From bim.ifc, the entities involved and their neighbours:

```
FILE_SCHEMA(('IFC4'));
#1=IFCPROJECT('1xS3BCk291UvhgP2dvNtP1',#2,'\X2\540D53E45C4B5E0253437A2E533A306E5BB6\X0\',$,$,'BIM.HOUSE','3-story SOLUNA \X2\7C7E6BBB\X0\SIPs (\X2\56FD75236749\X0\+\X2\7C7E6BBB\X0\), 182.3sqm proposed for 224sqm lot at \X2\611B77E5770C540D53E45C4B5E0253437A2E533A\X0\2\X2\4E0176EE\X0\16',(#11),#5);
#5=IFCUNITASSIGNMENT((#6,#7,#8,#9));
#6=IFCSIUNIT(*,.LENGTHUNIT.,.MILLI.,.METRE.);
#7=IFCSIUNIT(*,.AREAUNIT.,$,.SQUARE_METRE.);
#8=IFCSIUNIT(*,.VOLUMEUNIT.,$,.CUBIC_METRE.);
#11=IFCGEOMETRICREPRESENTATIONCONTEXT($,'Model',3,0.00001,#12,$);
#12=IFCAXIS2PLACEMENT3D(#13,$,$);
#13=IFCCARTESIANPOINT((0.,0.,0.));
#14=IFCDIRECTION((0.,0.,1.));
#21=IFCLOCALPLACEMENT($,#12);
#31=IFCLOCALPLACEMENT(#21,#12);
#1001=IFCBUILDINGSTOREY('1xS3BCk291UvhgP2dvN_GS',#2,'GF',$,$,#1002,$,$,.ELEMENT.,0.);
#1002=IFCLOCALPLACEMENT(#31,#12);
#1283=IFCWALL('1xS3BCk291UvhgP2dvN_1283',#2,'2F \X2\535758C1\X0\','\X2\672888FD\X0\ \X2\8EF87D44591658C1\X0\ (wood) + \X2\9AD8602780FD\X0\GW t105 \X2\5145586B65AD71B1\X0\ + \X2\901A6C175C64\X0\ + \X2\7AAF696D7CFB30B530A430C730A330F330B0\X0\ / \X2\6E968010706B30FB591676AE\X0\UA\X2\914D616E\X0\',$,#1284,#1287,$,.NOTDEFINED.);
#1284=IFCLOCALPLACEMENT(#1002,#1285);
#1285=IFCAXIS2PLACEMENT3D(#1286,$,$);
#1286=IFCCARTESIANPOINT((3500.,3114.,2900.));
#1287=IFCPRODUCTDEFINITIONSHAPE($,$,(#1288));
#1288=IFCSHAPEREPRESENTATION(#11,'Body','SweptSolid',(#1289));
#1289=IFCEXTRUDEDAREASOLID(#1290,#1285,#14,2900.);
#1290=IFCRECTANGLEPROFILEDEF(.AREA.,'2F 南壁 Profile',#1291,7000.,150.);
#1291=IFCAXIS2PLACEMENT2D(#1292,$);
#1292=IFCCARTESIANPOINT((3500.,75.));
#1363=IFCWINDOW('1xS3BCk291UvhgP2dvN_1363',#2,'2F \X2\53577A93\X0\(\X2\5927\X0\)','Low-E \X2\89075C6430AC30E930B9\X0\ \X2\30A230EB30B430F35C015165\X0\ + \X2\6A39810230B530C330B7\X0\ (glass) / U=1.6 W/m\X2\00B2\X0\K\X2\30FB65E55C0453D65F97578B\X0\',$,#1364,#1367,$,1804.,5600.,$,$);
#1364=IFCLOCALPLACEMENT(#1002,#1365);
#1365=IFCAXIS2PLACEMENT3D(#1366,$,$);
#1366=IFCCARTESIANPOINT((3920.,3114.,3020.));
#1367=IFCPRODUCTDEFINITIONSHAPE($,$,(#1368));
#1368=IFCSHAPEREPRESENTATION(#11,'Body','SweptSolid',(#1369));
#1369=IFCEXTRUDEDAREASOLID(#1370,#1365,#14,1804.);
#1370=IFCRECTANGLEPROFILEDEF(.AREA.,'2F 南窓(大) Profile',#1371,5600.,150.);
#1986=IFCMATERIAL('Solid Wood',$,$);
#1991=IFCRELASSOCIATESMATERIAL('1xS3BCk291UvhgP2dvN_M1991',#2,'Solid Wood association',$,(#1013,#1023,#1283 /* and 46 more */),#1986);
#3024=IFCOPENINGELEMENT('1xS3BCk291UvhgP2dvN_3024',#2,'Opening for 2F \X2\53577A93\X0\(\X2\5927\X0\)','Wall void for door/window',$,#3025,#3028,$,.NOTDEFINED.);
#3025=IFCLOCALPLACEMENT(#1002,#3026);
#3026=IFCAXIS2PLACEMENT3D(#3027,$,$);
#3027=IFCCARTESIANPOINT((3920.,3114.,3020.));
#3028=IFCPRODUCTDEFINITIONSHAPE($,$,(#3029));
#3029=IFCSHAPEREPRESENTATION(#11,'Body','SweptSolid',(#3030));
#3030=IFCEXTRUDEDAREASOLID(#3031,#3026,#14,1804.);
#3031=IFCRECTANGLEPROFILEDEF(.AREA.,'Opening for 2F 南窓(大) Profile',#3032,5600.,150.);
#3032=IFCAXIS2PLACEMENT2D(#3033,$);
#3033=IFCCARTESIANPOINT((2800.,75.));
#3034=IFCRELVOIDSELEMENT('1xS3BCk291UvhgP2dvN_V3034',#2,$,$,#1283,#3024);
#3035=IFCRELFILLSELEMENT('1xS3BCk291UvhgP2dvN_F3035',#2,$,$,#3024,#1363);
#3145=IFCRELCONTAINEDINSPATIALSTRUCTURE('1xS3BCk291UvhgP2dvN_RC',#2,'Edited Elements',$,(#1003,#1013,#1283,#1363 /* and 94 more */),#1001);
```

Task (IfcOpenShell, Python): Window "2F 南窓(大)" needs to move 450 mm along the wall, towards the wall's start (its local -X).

```python
import ifcopenshell
import ifcopenshell.api.geometry
import ifcopenshell.util.placement

model = ifcopenshell.open("bim.ifc")

window = model.by_id(1363)
opening = window.FillsVoids[0].RelatingOpeningElement
wall = opening.VoidsElements[0].RelatingBuildingElement

wall_matrix = ifcopenshell.util.placement.get_local_placement(wall.ObjectPlacement)
shift = wall_matrix[:3, 0] * -450.0
before = ifcopenshell.util.placement.get_local_placement(window.ObjectPlacement)[:3, 3].copy()

# The window is not placed relative to its opening, so move both.
for product in (opening, window):
    matrix = ifcopenshell.util.placement.get_local_placement(product.ObjectPlacement)
    matrix[:3, 3] += shift
    ifcopenshell.api.geometry.edit_object_placement(model, product=product, matrix=matrix, is_si=False)

after = ifcopenshell.util.placement.get_local_placement(window.ObjectPlacement)[:3, 3]
print("window moved by", (after - before).round(3) + 0.0)

model.write("bim_v2.ifc")
```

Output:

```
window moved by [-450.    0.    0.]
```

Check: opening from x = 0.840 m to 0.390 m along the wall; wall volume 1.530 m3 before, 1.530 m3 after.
